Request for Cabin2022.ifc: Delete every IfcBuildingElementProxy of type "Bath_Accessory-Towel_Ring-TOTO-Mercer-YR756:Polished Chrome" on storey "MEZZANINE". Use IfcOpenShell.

First a look at what the model holds.

```python
import ifcopenshell
import ifcopenshell.util.element

model = ifcopenshell.open("Cabin2022.ifc")
print(model.schema)
storey = next(s for s in model.by_type("IfcBuildingStorey") if s.Name == "MEZZANINE")
proxies = [e for e in ifcopenshell.util.element.get_decomposition(storey) if e.is_a("IfcBuildingElementProxy")]
seen = {}
for e in proxies:
    element_type = ifcopenshell.util.element.get_type(e)
    name = element_type.Name if element_type not in (None, e) else None
    seen[name] = seen.get(name, 0) + 1
for name, count in sorted(seen.items(), key=str):
    print(count, "x", name)
```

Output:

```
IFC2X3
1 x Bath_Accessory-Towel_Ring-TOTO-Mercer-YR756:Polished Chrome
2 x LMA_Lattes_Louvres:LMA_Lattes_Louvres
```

```python
import ifcopenshell
import ifcopenshell.api.root
import ifcopenshell.util.element

model = ifcopenshell.open("Cabin2022.ifc")

storey = next(s for s in model.by_type("IfcBuildingStorey") if s.Name == "MEZZANINE")
proxies = [e for e in ifcopenshell.util.element.get_decomposition(storey) if e.is_a("IfcBuildingElementProxy")]
targets = [e for e in proxies if (t := ifcopenshell.util.element.get_type(e)) not in (None, e) and t.Name == "Bath_Accessory-Towel_Ring-TOTO-Mercer-YR756:Polished Chrome"]

for e in targets:
    ifcopenshell.api.root.remove_product(model, product=e)
print(len(targets), "removed")

model.write("Cabin2022-out.ifc")
```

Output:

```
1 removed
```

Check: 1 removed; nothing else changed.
